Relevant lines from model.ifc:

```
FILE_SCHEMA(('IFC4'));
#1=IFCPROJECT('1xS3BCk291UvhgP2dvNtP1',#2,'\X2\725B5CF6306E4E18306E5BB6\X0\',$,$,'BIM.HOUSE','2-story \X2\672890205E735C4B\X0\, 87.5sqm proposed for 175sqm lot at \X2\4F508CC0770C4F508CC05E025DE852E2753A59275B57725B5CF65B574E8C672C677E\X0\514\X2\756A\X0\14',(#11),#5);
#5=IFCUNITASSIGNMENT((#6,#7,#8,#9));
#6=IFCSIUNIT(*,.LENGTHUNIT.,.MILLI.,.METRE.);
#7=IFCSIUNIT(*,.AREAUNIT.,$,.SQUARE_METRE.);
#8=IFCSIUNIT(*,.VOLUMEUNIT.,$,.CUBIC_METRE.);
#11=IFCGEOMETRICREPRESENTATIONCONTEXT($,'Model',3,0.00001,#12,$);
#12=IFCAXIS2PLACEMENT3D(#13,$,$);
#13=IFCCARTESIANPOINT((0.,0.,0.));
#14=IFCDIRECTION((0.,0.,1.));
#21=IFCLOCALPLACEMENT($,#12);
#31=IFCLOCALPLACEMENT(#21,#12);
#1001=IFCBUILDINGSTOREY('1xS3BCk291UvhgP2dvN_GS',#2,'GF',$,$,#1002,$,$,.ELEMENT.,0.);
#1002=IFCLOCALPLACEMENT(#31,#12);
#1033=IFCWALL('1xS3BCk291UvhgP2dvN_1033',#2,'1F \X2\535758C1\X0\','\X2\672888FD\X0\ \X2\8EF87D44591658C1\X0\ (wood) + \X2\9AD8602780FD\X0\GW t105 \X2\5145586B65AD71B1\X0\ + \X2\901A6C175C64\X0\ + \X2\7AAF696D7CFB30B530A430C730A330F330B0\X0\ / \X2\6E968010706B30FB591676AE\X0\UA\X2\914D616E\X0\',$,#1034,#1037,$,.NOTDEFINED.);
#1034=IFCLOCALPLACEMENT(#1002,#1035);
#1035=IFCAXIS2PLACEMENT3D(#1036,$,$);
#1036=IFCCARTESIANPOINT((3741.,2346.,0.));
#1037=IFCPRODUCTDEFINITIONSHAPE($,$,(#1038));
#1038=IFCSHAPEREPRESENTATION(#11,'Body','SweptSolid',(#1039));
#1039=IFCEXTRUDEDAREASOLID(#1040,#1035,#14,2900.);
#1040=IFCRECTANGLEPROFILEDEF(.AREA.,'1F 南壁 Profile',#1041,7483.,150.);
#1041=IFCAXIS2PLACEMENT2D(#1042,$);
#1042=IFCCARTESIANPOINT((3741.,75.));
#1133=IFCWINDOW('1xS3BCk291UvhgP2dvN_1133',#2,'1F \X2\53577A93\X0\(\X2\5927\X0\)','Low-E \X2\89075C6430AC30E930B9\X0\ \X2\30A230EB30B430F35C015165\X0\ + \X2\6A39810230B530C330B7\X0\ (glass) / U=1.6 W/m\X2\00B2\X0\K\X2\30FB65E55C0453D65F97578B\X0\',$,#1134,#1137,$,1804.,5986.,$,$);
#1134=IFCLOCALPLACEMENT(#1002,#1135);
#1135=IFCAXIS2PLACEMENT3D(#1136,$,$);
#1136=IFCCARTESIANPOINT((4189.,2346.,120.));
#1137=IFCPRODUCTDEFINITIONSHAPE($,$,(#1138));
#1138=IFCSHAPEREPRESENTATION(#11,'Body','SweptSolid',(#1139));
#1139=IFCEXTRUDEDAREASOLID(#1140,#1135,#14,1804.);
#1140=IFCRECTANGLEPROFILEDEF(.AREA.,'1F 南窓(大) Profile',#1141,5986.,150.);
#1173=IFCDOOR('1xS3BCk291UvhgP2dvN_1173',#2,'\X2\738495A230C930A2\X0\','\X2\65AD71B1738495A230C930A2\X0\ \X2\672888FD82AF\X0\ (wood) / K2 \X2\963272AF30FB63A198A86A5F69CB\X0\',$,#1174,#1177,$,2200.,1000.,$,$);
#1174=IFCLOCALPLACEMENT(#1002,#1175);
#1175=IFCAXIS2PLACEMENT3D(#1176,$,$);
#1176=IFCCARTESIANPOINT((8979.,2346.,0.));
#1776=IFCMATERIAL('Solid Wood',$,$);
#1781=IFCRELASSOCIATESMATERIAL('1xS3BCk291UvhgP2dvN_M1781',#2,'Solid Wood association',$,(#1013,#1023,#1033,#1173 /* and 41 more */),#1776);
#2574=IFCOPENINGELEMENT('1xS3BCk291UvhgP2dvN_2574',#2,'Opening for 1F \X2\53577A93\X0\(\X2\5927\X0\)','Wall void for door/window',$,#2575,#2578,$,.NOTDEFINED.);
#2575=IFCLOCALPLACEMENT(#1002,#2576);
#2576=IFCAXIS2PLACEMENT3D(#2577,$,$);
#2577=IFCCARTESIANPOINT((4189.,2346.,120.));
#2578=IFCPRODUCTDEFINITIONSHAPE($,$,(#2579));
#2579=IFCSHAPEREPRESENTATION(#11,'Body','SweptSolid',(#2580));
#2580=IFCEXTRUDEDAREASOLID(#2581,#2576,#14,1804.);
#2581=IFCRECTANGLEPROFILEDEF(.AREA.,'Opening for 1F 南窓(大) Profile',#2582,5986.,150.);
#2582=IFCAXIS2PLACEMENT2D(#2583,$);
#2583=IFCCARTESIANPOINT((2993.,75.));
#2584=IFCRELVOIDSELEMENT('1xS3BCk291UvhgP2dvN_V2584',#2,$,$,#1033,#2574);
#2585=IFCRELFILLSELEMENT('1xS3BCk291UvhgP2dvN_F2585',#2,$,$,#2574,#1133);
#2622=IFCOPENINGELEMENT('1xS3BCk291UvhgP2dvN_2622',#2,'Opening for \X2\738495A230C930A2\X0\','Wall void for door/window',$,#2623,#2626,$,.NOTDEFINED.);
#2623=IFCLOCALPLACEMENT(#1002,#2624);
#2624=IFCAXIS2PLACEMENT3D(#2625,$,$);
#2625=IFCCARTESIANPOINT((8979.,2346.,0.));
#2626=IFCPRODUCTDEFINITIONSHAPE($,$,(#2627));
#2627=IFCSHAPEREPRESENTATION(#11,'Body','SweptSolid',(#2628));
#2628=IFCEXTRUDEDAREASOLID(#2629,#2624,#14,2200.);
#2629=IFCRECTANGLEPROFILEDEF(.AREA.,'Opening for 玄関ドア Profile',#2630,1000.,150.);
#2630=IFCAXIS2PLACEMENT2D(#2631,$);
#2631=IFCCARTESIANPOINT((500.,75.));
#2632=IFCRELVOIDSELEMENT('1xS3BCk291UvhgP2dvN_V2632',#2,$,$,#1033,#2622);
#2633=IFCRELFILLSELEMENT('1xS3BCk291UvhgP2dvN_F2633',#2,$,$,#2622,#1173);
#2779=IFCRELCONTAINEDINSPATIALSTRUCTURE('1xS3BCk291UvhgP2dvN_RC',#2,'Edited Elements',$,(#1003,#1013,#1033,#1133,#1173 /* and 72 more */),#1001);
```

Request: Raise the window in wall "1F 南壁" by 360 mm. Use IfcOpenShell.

```python
import numpy as np
import ifcopenshell
import ifcopenshell.api.geometry
import ifcopenshell.util.placement
import ifcopenshell.util.unit

model = ifcopenshell.open("model.ifc")
unit_scale = ifcopenshell.util.unit.calculate_unit_scale(model)

window = model.by_guid("1xS3BCk291UvhgP2dvN_1133")
opening = window.FillsVoids[0].RelatingOpeningElement
dz = 0.36 / unit_scale

shift = np.array([0.0, 0.0, dz])
# The window is not placed relative to its opening, so move both.
for product in (opening, window):
    matrix = ifcopenshell.util.placement.get_local_placement(product.ObjectPlacement)
    matrix[:3, 3] += shift
    ifcopenshell.api.geometry.edit_object_placement(model, product=product, matrix=matrix, is_si=False)

print(f"moved by {dz * unit_scale:+.3f} m")

model.write("model_v2.ifc")
```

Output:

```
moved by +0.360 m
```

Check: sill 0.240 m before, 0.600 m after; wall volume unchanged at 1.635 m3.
